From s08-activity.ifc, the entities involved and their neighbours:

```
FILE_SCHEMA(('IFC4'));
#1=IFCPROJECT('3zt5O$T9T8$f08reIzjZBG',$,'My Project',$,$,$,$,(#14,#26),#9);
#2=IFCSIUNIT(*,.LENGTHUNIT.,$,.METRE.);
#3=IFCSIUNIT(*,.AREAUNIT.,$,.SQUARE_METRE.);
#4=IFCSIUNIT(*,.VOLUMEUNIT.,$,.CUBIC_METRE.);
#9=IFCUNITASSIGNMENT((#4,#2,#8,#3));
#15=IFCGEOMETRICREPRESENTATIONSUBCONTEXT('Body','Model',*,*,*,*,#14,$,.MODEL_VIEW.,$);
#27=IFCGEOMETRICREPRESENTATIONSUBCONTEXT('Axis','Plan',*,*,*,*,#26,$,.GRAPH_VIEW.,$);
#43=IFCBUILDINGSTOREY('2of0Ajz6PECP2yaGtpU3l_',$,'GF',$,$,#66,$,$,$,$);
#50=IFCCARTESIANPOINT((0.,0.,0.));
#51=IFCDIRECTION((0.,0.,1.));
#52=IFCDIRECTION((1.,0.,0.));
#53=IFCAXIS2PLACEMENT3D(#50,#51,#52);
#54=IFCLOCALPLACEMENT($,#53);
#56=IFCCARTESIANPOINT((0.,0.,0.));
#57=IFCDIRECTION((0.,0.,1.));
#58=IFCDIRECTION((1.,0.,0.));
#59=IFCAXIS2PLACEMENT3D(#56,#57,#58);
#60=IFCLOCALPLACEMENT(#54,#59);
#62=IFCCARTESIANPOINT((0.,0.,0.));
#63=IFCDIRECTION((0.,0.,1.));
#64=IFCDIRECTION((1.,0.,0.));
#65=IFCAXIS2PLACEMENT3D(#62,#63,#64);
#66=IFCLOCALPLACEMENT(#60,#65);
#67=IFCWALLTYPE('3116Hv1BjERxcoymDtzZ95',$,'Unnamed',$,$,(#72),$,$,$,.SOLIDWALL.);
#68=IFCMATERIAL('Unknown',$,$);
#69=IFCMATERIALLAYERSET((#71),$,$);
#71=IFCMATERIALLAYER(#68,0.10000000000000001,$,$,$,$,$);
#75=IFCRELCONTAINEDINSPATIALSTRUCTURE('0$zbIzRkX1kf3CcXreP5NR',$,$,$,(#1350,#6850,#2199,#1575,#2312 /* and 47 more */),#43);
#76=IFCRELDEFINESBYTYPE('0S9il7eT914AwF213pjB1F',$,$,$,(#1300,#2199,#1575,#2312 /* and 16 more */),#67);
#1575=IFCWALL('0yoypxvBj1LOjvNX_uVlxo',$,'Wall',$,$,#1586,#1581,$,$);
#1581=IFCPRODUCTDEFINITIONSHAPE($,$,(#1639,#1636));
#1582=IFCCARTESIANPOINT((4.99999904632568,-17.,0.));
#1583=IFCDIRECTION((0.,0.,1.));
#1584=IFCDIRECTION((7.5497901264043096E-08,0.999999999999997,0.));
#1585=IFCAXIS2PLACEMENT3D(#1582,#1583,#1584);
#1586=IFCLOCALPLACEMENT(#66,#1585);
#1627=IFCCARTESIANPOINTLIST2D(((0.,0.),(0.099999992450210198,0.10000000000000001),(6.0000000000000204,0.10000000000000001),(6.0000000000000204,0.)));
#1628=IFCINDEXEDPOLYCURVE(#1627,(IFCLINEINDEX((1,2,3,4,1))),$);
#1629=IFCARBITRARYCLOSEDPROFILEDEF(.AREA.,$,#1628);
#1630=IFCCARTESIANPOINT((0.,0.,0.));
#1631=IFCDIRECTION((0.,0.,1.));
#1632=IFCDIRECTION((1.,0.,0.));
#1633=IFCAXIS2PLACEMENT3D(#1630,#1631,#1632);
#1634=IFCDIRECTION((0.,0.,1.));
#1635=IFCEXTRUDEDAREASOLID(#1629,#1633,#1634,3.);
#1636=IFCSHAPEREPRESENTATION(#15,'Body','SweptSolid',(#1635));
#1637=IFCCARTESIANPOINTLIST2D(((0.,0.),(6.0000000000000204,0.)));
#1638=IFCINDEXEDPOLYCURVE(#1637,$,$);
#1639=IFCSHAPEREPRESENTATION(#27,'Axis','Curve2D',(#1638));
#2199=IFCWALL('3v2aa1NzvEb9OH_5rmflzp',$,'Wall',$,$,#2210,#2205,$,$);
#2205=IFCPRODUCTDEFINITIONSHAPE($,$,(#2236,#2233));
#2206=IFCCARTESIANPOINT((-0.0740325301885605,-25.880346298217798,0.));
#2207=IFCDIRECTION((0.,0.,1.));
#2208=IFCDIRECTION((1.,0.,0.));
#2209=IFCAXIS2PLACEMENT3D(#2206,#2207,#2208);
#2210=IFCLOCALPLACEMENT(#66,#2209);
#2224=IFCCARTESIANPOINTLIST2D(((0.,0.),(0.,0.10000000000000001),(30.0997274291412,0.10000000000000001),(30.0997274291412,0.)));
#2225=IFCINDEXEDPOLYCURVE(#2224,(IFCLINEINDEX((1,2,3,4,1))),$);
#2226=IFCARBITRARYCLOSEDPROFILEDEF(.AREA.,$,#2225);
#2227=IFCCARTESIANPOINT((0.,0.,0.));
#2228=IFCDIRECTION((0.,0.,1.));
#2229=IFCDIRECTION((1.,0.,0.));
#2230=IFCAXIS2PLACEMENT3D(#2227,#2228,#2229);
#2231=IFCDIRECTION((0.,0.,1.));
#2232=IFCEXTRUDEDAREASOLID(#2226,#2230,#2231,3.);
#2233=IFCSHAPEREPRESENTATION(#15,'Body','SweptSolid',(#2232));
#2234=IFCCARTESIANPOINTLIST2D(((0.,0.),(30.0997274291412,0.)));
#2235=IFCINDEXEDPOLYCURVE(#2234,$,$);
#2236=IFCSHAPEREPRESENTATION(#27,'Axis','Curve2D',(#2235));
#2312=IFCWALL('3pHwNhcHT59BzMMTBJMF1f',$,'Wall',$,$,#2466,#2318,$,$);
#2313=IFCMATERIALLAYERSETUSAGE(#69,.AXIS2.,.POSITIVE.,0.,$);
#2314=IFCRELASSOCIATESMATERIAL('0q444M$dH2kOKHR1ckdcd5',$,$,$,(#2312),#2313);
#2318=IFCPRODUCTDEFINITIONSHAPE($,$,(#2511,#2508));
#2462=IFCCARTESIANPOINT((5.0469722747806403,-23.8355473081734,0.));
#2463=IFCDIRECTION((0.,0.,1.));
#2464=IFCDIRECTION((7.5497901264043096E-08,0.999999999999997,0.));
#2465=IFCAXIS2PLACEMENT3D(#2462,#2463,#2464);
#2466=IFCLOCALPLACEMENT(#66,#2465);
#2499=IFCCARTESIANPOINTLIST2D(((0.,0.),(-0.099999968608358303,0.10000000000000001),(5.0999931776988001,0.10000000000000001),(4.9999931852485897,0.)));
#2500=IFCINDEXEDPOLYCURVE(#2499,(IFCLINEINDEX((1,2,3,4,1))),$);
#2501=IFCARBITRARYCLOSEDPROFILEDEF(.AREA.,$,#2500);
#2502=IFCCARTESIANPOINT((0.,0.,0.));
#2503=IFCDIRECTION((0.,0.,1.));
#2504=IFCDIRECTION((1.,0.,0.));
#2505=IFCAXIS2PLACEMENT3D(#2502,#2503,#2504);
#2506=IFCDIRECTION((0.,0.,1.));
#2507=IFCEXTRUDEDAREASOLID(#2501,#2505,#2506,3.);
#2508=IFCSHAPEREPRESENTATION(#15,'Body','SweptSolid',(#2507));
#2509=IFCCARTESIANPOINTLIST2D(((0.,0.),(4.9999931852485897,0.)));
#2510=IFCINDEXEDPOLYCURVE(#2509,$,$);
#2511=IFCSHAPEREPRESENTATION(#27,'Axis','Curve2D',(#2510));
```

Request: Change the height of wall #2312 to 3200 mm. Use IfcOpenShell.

```python
import ifcopenshell
import ifcopenshell.geom
import ifcopenshell.util.representation
import ifcopenshell.util.shape
import ifcopenshell.util.unit

model = ifcopenshell.open("s08-activity.ifc")
unit_scale = ifcopenshell.util.unit.calculate_unit_scale(model)
settings = ifcopenshell.geom.settings()


def volume(element):
    """Net volume in cubic metres, openings subtracted."""
    shape = ifcopenshell.geom.create_shape(settings, element)
    return ifcopenshell.util.shape.get_volume(shape.geometry)


wall = model.by_id(2312)
before = volume(wall)

body = ifcopenshell.util.representation.get_representation(wall, "Model", "Body")
solid = body.Items[0]
old_height = solid.Depth
solid.Depth = 3.2 / unit_scale
after = volume(wall)

print(f"height {old_height:g} -> {solid.Depth:g}, volume {before:.3f} -> {after:.3f} m3")

model.write("s08-activity_updated.ifc")
```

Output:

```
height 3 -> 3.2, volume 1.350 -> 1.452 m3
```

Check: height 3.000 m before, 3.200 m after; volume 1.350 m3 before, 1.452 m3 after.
